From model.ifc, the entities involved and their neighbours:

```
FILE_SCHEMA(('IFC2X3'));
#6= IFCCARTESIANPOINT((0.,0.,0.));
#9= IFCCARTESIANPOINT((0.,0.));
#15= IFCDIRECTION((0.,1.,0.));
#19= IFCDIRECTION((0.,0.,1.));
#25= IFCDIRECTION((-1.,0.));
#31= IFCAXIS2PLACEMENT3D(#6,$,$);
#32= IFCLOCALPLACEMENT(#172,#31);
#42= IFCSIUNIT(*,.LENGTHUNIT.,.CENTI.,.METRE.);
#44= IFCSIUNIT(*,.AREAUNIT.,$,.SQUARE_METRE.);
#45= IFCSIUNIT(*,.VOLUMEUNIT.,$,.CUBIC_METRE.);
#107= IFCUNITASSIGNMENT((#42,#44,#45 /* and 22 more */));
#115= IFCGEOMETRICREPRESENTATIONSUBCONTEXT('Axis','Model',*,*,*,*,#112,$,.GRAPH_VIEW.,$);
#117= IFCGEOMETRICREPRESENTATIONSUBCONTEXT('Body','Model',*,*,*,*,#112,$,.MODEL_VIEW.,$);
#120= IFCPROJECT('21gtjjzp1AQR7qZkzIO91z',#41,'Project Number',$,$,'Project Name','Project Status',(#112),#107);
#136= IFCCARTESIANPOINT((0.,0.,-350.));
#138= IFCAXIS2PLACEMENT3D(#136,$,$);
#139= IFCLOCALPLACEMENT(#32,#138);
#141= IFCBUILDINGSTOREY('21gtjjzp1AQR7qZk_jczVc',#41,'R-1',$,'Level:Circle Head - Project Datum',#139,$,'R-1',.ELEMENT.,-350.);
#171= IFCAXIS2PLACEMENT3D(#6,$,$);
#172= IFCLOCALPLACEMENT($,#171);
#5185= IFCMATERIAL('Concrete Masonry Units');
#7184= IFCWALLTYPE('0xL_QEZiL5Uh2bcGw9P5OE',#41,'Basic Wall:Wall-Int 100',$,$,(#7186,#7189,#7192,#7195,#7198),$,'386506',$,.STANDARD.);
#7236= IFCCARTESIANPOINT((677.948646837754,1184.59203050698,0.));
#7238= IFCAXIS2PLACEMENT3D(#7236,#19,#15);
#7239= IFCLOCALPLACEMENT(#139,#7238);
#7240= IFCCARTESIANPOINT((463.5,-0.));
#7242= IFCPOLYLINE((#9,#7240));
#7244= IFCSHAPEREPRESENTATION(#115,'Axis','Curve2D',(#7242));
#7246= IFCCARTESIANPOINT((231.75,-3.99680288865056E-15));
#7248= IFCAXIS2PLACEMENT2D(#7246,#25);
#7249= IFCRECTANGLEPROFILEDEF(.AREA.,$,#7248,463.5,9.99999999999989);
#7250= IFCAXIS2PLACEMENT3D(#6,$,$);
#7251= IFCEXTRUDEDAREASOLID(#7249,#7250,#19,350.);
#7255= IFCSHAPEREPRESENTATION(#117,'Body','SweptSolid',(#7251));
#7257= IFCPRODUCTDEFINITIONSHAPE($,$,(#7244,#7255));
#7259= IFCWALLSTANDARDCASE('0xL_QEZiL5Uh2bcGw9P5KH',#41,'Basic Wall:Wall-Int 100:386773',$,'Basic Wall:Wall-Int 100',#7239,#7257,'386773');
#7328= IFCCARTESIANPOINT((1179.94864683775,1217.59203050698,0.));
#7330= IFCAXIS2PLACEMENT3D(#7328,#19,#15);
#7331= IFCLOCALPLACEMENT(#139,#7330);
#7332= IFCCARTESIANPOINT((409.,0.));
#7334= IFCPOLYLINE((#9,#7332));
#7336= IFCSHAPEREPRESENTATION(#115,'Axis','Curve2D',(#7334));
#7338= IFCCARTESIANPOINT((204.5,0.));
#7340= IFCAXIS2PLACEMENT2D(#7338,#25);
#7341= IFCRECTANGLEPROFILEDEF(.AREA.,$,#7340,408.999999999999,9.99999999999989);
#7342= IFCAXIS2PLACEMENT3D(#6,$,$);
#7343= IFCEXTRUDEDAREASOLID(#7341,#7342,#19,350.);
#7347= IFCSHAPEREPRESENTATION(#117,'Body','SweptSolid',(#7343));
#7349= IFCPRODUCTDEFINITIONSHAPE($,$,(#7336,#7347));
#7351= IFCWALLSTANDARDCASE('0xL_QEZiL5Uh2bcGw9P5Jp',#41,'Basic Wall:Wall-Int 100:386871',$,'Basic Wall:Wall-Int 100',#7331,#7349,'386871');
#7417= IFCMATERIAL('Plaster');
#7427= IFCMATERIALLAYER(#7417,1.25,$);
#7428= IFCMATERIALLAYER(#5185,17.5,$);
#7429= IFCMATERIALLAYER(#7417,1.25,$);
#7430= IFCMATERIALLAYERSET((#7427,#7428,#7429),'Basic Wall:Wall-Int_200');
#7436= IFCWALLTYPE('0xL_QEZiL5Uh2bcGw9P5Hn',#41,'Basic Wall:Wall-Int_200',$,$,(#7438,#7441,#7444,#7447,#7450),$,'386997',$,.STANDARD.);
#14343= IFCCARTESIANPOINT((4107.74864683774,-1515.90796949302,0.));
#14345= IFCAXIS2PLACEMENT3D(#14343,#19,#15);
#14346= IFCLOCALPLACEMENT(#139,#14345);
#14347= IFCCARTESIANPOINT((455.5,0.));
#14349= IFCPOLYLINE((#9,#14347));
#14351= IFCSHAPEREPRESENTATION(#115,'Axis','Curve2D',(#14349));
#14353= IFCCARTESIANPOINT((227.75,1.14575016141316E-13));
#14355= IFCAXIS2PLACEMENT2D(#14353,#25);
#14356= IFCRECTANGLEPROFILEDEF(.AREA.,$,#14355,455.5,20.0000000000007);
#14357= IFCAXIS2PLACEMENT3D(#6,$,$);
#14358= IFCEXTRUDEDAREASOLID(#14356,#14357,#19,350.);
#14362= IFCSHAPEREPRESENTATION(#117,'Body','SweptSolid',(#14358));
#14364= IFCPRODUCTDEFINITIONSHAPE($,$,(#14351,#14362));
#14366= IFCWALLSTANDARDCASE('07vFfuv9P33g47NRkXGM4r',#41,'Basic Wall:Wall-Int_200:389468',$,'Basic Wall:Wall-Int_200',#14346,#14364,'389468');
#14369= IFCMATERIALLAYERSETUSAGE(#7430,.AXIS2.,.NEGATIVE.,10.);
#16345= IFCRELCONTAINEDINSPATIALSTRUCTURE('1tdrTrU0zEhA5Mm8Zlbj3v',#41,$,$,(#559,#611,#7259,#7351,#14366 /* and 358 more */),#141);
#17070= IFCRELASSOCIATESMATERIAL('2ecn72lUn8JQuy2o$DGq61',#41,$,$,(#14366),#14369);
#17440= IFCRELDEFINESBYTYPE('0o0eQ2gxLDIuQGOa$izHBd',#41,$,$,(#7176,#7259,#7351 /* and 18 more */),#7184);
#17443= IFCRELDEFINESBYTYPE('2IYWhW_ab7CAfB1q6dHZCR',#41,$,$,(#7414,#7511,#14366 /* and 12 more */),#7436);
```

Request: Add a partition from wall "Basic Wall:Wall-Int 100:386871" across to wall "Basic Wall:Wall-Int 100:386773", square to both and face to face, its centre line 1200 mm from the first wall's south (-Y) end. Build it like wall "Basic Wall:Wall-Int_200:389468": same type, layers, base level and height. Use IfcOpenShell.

```python
import numpy as np
import ifcopenshell
import ifcopenshell.api.geometry
import ifcopenshell.api.material
import ifcopenshell.api.pset
import ifcopenshell.api.root
import ifcopenshell.api.spatial
import ifcopenshell.api.type
import ifcopenshell.geom
import ifcopenshell.util.element
import ifcopenshell.util.placement
import ifcopenshell.util.representation
import ifcopenshell.util.shape
import ifcopenshell.util.unit

model = ifcopenshell.open("model.ifc")
unit_scale = ifcopenshell.util.unit.calculate_unit_scale(model)
settings = ifcopenshell.geom.settings()
settings.set("use-world-coords", True)

start_wall = model.by_id(7351)
end_wall = model.by_guid("0xL_QEZiL5Uh2bcGw9P5KH")
like = model.by_guid("07vFfuv9P33g47NRkXGM4r")
matrix = ifcopenshell.util.placement.get_local_placement(start_wall.ObjectPlacement)
matrix[:3, 3] *= unit_scale


def extent(element):
    """Bounding box in the first wall's axes, in metres."""
    shape = ifcopenshell.geom.create_shape(settings, element)
    points = (ifcopenshell.util.shape.get_vertices(shape.geometry) - matrix[:3, 3]) @ matrix[:3, :3]
    return points.min(axis=0), points.max(axis=0)


y_start = extent(start_wall)[1][1]
y_end = extent(end_wall)[0][1]
like_min, like_max = extent(like)
length, height = float(abs(y_end - y_start)), float(like_max[2] - like_min[2])
layer_set = ifcopenshell.util.element.get_material(like, should_skip_usage=True)
thickness = sum(layer.LayerThickness for layer in layer_set.MaterialLayers) * unit_scale

wall = ifcopenshell.api.root.create_entity(model, ifc_class="IfcWallStandardCase", name="New partition")
storey = ifcopenshell.util.element.get_container(like)
ifcopenshell.api.spatial.assign_container(model, products=[wall], relating_structure=storey)
ifcopenshell.api.type.assign_type(
    model, related_objects=[wall], relating_type=ifcopenshell.util.element.get_type(like), should_map_representations=False
)
rel = ifcopenshell.api.material.assign_material(
    model, products=[wall], type="IfcMaterialLayerSetUsage", material=layer_set
)
rel.RelatingMaterial.OffsetFromReferenceLine = -thickness / 2 / unit_scale
pset = ifcopenshell.api.pset.add_pset(model, product=wall, name="Pset_WallCommon")
ifcopenshell.api.pset.edit_pset(model, pset=pset, properties={"IsExternal": False, "LoadBearing": False})

# The axis runs down the middle of the wall.
axis = ifcopenshell.api.geometry.add_axis_representation(
    model, context=ifcopenshell.util.representation.get_context(model, "Model", "Axis"), axis=[(0.0, 0.0), (length, 0.0)]
)
body = ifcopenshell.api.geometry.add_wall_representation(
    model,
    context=ifcopenshell.util.representation.get_context(model, "Model", "Body", "MODEL_VIEW"),
    length=length,
    height=height,
    thickness=thickness,
    offset=-thickness / 2,
)
for representation in (axis, body):
    ifcopenshell.api.geometry.assign_representation(model, product=wall, representation=representation)

placement = matrix @ ifcopenshell.util.placement.rotation(90, "Z")
placement[:, 3] = matrix @ np.array([extent(start_wall)[0][0] + 1.2, y_start, like_min[2], 1.0])
ifcopenshell.api.geometry.edit_object_placement(model, product=wall, matrix=placement)

print(f"partition {length:.3f} m long, {height:.3f} m high, {thickness:.3f} m thick")

model.write("model_rev.ifc")
```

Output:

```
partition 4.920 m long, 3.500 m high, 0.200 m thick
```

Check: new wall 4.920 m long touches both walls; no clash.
